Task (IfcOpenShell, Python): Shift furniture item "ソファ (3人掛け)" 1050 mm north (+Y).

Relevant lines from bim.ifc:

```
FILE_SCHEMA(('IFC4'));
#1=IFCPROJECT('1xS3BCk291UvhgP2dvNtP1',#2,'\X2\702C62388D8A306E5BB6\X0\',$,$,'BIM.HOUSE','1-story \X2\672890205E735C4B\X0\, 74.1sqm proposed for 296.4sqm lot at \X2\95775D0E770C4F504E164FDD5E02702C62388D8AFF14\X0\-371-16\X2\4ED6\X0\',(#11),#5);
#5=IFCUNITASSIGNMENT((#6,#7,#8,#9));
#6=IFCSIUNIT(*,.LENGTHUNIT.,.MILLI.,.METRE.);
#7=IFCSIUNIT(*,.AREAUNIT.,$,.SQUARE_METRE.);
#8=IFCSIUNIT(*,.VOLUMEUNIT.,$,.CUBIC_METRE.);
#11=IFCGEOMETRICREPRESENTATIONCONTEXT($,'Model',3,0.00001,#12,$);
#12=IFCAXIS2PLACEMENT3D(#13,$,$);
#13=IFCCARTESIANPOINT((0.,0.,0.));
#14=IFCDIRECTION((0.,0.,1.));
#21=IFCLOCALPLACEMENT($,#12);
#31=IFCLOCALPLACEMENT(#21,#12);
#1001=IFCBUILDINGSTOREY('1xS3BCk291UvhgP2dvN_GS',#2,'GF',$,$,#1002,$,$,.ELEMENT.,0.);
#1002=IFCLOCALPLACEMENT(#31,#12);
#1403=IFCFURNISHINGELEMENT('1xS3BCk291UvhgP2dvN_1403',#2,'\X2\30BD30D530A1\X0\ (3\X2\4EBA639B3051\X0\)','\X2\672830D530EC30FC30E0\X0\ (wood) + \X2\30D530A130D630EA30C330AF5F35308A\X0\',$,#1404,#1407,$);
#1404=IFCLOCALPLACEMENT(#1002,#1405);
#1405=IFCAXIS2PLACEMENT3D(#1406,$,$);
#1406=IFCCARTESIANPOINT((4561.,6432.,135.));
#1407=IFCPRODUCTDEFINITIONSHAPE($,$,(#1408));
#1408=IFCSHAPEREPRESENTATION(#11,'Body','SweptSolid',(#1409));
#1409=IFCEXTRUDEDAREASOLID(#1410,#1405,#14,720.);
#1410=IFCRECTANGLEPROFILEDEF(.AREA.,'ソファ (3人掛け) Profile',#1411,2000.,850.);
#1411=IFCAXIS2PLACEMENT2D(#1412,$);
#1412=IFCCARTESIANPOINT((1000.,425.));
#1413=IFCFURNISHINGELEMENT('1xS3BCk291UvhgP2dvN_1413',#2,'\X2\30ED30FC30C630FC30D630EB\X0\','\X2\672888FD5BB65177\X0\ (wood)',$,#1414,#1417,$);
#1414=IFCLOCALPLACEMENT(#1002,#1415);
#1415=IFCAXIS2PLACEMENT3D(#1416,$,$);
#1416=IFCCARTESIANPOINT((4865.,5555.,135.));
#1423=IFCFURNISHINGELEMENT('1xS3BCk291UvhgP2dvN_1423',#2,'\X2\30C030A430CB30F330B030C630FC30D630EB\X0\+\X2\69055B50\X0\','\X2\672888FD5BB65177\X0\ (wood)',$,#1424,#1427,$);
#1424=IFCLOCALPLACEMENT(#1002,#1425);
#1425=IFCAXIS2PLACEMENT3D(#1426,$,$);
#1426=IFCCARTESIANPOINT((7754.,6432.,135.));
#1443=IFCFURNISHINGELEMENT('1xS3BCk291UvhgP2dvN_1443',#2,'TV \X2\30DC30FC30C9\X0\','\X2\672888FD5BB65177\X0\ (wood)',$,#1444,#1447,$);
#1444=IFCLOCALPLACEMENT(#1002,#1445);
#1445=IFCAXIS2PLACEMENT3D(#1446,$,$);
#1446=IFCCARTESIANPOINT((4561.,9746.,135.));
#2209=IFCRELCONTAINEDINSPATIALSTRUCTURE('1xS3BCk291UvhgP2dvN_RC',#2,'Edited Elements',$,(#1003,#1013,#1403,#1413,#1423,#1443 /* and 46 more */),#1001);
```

```python
import ifcopenshell
import ifcopenshell.api.geometry
import ifcopenshell.util.placement

model = ifcopenshell.open("bim.ifc")

item = model.by_guid("1xS3BCk291UvhgP2dvN_1403")
matrix = ifcopenshell.util.placement.get_local_placement(item.ObjectPlacement)
matrix[1, 3] += 1050.0
ifcopenshell.api.geometry.edit_object_placement(model, product=item, matrix=matrix, is_si=False)

print(ifcopenshell.util.placement.get_local_placement(item.ObjectPlacement).round(3) + 0.0)

model.write("bim_updated.ifc")
```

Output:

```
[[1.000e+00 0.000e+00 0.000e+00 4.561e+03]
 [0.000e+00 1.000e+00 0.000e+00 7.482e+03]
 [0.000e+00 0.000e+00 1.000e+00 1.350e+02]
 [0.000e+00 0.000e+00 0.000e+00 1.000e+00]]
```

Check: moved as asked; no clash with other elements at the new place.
